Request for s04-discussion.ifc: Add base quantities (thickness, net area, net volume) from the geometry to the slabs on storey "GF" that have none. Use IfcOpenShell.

First a look at what the model holds.

```python
import ifcopenshell
import ifcopenshell.util.element
import ifcopenshell.util.unit

model = ifcopenshell.open("s04-discussion.ifc")
print(model.schema)
for unit_type in ("LENGTHUNIT", "AREAUNIT", "VOLUMEUNIT"):
    print(unit_type, ifcopenshell.util.unit.calculate_unit_scale(model, unit_type))
storey = next(s for s in model.by_type("IfcBuildingStorey") if s.Name == "GF")
slabs = [e for e in ifcopenshell.util.element.get_decomposition(storey) if e.is_a("IfcSlab")]
for e in sorted(slabs, key=lambda e: e.id()):
    print(e.id(), e.is_a(), e.Name, list(ifcopenshell.util.element.get_psets(e, qtos_only=True)), sep=" | ")
```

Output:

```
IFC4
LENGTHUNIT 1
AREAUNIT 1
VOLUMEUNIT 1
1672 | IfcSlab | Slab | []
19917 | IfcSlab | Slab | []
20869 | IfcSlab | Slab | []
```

```python
import ifcopenshell
import ifcopenshell.api.pset
import ifcopenshell.geom
import ifcopenshell.util.element
import ifcopenshell.util.shape
import ifcopenshell.util.unit

model = ifcopenshell.open("s04-discussion.ifc")
unit_scale = ifcopenshell.util.unit.calculate_unit_scale(model)
area_scale = ifcopenshell.util.unit.calculate_unit_scale(model, "AREAUNIT")
volume_scale = ifcopenshell.util.unit.calculate_unit_scale(model, "VOLUMEUNIT")
settings = ifcopenshell.geom.settings()

storey = next(s for s in model.by_type("IfcBuildingStorey") if s.Name == "GF")
slabs = [e for e in ifcopenshell.util.element.get_decomposition(storey) if e.is_a("IfcSlab")]

for e in sorted(slabs, key=lambda e: e.id()):
    if ifcopenshell.util.element.get_psets(e, qtos_only=True, should_inherit=False):
        continue
    # Geometry comes back in metres, in the element's own axes.
    shape = ifcopenshell.geom.create_shape(settings, e)
    values = {
        "Width": ifcopenshell.util.shape.get_z(shape.geometry) / unit_scale,
        "NetArea": ifcopenshell.util.shape.get_footprint_area(shape.geometry) / area_scale,
        "NetVolume": ifcopenshell.util.shape.get_volume(shape.geometry) / volume_scale,
    }
    qto = ifcopenshell.api.pset.add_qto(model, product=e, name="Qto_SlabBaseQuantities")
    ifcopenshell.api.pset.edit_qto(model, qto=qto, properties=values)
    print(e.id(), {k: round(v, 3) for k, v in values.items()})

model.write("s04-discussion_rev.ifc")
```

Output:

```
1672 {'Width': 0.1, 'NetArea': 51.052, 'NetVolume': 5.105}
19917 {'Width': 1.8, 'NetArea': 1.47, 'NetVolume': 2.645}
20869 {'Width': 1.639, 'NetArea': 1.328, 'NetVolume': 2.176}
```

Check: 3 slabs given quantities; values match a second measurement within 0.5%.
